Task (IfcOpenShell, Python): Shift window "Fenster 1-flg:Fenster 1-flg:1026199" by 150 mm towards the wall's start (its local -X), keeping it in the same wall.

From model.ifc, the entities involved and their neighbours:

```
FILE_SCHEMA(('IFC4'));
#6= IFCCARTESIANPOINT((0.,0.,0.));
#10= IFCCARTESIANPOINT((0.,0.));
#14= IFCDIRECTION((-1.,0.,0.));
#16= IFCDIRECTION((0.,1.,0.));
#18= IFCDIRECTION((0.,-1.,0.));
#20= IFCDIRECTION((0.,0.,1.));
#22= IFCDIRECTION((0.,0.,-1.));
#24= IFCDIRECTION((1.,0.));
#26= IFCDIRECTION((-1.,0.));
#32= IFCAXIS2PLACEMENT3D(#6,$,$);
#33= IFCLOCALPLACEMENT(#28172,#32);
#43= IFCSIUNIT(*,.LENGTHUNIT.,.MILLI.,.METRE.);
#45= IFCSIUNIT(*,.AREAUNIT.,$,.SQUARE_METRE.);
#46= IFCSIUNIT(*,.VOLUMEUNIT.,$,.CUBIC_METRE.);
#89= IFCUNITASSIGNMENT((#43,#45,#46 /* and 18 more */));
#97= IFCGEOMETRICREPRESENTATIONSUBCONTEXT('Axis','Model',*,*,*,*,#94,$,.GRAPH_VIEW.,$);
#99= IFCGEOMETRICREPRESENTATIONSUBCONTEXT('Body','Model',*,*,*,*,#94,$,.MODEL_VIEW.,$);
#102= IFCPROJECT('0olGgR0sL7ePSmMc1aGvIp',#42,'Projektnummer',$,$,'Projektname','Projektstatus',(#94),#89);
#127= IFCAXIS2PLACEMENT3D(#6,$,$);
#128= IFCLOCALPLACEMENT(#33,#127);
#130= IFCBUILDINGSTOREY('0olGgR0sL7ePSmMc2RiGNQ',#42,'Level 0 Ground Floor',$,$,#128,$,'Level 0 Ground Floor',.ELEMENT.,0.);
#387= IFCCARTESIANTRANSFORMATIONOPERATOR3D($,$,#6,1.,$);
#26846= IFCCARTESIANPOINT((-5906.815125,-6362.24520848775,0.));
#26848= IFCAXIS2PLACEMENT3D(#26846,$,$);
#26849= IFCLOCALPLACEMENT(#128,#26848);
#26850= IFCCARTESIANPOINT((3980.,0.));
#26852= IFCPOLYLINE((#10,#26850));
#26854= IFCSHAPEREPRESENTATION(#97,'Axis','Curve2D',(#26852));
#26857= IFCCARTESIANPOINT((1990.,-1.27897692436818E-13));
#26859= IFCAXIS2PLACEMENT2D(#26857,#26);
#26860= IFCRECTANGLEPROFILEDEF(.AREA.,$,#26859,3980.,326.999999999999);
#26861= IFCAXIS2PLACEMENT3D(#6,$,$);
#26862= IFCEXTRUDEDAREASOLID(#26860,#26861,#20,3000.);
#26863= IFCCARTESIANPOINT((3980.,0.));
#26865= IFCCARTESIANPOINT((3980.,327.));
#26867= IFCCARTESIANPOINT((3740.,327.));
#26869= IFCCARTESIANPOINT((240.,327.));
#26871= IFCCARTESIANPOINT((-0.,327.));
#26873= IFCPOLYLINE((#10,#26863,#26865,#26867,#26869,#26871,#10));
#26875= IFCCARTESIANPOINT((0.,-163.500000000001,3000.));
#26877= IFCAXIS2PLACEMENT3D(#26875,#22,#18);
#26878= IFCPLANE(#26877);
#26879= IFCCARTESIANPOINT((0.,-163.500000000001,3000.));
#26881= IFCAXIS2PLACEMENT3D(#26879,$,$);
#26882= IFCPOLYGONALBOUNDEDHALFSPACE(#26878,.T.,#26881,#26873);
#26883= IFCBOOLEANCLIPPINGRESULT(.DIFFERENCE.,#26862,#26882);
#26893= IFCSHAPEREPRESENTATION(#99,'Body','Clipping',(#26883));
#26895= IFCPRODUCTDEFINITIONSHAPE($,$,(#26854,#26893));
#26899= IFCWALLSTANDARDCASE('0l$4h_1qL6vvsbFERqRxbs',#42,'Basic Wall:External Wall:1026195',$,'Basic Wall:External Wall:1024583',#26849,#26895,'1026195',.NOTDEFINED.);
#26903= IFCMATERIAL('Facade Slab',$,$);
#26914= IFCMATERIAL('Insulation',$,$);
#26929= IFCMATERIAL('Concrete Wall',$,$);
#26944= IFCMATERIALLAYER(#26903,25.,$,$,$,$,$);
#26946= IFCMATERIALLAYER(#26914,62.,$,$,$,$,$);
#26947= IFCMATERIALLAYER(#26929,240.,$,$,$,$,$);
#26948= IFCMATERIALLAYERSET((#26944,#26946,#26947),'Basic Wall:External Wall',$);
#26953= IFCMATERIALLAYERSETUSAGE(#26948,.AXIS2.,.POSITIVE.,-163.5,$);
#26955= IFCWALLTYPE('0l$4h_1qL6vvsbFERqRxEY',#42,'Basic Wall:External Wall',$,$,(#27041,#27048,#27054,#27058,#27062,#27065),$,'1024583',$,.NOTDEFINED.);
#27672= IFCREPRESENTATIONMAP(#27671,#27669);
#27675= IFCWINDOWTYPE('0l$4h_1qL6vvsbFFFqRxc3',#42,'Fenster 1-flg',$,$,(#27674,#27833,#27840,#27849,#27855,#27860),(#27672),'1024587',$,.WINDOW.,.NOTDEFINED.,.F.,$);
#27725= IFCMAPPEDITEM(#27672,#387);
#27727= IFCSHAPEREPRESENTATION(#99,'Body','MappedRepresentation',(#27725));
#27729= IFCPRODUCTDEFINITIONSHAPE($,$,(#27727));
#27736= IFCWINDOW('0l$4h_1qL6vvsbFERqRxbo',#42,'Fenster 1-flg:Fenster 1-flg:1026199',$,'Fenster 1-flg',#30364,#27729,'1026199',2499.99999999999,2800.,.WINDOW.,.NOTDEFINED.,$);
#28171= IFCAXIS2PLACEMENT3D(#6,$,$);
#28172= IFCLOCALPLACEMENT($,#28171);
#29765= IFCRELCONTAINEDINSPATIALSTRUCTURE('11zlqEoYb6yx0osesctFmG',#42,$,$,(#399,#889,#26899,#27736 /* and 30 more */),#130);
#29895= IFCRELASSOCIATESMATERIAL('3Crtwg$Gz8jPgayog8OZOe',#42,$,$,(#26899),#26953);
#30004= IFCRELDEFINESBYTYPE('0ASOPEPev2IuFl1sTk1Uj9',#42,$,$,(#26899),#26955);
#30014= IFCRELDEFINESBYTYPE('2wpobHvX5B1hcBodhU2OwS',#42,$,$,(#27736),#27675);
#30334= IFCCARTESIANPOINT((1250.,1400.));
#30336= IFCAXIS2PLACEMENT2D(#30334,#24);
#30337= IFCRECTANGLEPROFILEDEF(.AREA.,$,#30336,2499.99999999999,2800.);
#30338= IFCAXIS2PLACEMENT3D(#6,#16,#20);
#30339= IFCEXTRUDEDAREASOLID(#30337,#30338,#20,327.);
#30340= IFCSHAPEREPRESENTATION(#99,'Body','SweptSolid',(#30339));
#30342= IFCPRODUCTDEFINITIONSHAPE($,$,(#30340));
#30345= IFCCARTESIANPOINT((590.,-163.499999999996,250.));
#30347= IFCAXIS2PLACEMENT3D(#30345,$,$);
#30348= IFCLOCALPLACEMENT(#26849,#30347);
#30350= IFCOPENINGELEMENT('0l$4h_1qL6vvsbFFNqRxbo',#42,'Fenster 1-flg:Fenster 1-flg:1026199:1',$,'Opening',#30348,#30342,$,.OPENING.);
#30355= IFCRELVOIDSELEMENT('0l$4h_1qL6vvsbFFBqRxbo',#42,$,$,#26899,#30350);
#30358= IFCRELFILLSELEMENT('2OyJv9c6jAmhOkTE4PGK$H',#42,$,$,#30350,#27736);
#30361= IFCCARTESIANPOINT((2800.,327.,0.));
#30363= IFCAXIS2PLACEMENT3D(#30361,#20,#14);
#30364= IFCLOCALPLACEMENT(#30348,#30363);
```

```python
import ifcopenshell
import ifcopenshell.api.geometry
import ifcopenshell.util.placement
import ifcopenshell.util.unit

model = ifcopenshell.open("model.ifc")
unit_scale = ifcopenshell.util.unit.calculate_unit_scale(model)

window = model.by_id(27736)
opening = window.FillsVoids[0].RelatingOpeningElement
wall = opening.VoidsElements[0].RelatingBuildingElement

wall_matrix = ifcopenshell.util.placement.get_local_placement(wall.ObjectPlacement)
shift = wall_matrix[:3, 0] * -0.15 / unit_scale
before = ifcopenshell.util.placement.get_local_placement(window.ObjectPlacement)[:3, 3].copy()

# The window is placed relative to its opening, so it follows when the opening moves.
matrix = ifcopenshell.util.placement.get_local_placement(opening.ObjectPlacement)
matrix[:3, 3] += shift
ifcopenshell.api.geometry.edit_object_placement(
    model, product=opening, matrix=matrix, is_si=False, should_transform_children=True
)

after = ifcopenshell.util.placement.get_local_placement(window.ObjectPlacement)[:3, 3]
print("window moved by", (after - before).round(3) + 0.0)

model.write("model_updated.ifc")
```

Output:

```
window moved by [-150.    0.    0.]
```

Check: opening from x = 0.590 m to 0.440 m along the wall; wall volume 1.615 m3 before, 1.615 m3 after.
